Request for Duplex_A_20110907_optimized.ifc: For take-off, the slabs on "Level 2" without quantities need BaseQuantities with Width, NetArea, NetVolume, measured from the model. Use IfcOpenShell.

First a look at what the model holds.

```python
import ifcopenshell
import ifcopenshell.util.element
import ifcopenshell.util.unit

model = ifcopenshell.open("Duplex_A_20110907_optimized.ifc")
print(model.schema)
for unit_type in ("LENGTHUNIT", "AREAUNIT", "VOLUMEUNIT"):
    print(unit_type, ifcopenshell.util.unit.calculate_unit_scale(model, unit_type))
storey = next(s for s in model.by_type("IfcBuildingStorey") if s.Name == "Level 2")
slabs = [e for e in ifcopenshell.util.element.get_decomposition(storey) if e.is_a("IfcSlab")]
for e in sorted(slabs, key=lambda e: e.id()):
    print(e.id(), e.is_a(), e.Name, list(ifcopenshell.util.element.get_psets(e, qtos_only=True)), sep=" | ")
```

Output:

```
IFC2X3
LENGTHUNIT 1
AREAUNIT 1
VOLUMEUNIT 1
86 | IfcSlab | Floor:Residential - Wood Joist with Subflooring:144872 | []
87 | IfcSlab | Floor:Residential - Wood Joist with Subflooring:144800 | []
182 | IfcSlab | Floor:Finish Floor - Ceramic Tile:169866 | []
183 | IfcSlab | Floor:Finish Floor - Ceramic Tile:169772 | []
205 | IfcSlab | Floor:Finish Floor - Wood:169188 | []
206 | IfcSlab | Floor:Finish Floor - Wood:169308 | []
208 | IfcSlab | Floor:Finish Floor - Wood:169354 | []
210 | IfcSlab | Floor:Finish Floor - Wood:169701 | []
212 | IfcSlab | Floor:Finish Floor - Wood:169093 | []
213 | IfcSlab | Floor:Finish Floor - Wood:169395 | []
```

```python
import ifcopenshell
import ifcopenshell.api.pset
import ifcopenshell.geom
import ifcopenshell.util.element
import ifcopenshell.util.shape
import ifcopenshell.util.unit

model = ifcopenshell.open("Duplex_A_20110907_optimized.ifc")
unit_scale = ifcopenshell.util.unit.calculate_unit_scale(model)
area_scale = ifcopenshell.util.unit.calculate_unit_scale(model, "AREAUNIT")
volume_scale = ifcopenshell.util.unit.calculate_unit_scale(model, "VOLUMEUNIT")
settings = ifcopenshell.geom.settings()

storey = next(s for s in model.by_type("IfcBuildingStorey") if s.Name == "Level 2")
slabs = [e for e in ifcopenshell.util.element.get_decomposition(storey) if e.is_a("IfcSlab")]

for e in sorted(slabs, key=lambda e: e.id()):
    if ifcopenshell.util.element.get_psets(e, qtos_only=True, should_inherit=False):
        continue
    # Geometry comes back in metres, in the element's own axes.
    shape = ifcopenshell.geom.create_shape(settings, e)
    values = {
        "Width": ifcopenshell.util.shape.get_z(shape.geometry) / unit_scale,
        "NetArea": ifcopenshell.util.shape.get_footprint_area(shape.geometry) / area_scale,
        "NetVolume": ifcopenshell.util.shape.get_volume(shape.geometry) / volume_scale,
    }
    qto = ifcopenshell.api.pset.add_qto(model, product=e, name="BaseQuantities")
    ifcopenshell.api.pset.edit_qto(model, qto=qto, properties=values)
    print(e.id(), {k: round(v, 3) for k, v in values.items()})

model.write("Duplex_A_20110907_optimized_rev.ifc")
```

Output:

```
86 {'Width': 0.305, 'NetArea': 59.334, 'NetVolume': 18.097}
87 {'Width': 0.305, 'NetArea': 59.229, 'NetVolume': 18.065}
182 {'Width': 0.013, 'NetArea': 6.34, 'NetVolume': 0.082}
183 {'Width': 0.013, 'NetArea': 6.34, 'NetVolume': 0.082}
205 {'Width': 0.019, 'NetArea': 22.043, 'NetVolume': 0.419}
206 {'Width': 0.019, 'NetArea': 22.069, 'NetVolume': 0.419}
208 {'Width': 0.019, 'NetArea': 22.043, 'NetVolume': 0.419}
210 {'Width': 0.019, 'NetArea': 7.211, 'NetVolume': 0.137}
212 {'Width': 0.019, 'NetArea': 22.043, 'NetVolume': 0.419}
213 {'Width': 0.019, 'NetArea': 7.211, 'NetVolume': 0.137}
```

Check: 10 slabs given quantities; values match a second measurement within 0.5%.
